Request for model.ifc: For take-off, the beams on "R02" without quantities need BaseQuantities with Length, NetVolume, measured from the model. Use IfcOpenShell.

First a look at what the model holds.

```python
import ifcopenshell
import ifcopenshell.util.element
import ifcopenshell.util.unit

model = ifcopenshell.open("model.ifc")
print(model.schema)
for unit_type in ("LENGTHUNIT", "AREAUNIT", "VOLUMEUNIT"):
    print(unit_type, ifcopenshell.util.unit.calculate_unit_scale(model, unit_type))
storey = next(s for s in model.by_type("IfcBuildingStorey") if s.Name == "R02")
beams = [e for e in ifcopenshell.util.element.get_decomposition(storey) if e.is_a("IfcBeam")]
for e in sorted(beams, key=lambda e: e.id()):
    print(e.id(), e.is_a(), e.Name, list(ifcopenshell.util.element.get_psets(e, qtos_only=True)), sep=" | ")
```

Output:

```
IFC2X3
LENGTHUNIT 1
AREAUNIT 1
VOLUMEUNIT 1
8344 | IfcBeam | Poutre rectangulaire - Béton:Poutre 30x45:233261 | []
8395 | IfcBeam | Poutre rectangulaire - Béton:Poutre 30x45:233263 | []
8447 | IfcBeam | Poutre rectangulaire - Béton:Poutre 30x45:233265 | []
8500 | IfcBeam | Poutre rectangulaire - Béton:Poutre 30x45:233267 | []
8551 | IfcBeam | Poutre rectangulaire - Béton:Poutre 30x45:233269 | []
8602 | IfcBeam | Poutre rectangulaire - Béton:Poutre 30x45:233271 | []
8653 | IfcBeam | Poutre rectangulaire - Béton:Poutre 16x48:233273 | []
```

```python
import ifcopenshell
import ifcopenshell.api.pset
import ifcopenshell.geom
import ifcopenshell.util.element
import ifcopenshell.util.shape
import ifcopenshell.util.unit

model = ifcopenshell.open("model.ifc")
unit_scale = ifcopenshell.util.unit.calculate_unit_scale(model)
volume_scale = ifcopenshell.util.unit.calculate_unit_scale(model, "VOLUMEUNIT")
settings = ifcopenshell.geom.settings()

storey = next(s for s in model.by_type("IfcBuildingStorey") if s.Name == "R02")
beams = [e for e in ifcopenshell.util.element.get_decomposition(storey) if e.is_a("IfcBeam")]

for e in sorted(beams, key=lambda e: e.id()):
    if ifcopenshell.util.element.get_psets(e, qtos_only=True, should_inherit=False):
        continue
    # Geometry comes back in metres, in the element's own axes.
    shape = ifcopenshell.geom.create_shape(settings, e)
    values = {
        "Length": ifcopenshell.util.shape.get_max_xyz(shape.geometry) / unit_scale,
        "NetVolume": ifcopenshell.util.shape.get_volume(shape.geometry) / volume_scale,
    }
    qto = ifcopenshell.api.pset.add_qto(model, product=e, name="BaseQuantities")
    ifcopenshell.api.pset.edit_qto(model, qto=qto, properties=values)
    print(e.id(), {k: round(v, 3) for k, v in values.items()})

model.write("model-out.ifc")
```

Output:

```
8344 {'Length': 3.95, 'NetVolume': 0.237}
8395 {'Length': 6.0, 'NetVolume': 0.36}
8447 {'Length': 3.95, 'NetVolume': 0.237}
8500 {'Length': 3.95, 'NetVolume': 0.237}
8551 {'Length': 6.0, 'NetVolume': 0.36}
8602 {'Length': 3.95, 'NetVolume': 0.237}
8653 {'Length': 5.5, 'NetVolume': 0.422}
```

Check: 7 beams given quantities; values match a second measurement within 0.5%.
